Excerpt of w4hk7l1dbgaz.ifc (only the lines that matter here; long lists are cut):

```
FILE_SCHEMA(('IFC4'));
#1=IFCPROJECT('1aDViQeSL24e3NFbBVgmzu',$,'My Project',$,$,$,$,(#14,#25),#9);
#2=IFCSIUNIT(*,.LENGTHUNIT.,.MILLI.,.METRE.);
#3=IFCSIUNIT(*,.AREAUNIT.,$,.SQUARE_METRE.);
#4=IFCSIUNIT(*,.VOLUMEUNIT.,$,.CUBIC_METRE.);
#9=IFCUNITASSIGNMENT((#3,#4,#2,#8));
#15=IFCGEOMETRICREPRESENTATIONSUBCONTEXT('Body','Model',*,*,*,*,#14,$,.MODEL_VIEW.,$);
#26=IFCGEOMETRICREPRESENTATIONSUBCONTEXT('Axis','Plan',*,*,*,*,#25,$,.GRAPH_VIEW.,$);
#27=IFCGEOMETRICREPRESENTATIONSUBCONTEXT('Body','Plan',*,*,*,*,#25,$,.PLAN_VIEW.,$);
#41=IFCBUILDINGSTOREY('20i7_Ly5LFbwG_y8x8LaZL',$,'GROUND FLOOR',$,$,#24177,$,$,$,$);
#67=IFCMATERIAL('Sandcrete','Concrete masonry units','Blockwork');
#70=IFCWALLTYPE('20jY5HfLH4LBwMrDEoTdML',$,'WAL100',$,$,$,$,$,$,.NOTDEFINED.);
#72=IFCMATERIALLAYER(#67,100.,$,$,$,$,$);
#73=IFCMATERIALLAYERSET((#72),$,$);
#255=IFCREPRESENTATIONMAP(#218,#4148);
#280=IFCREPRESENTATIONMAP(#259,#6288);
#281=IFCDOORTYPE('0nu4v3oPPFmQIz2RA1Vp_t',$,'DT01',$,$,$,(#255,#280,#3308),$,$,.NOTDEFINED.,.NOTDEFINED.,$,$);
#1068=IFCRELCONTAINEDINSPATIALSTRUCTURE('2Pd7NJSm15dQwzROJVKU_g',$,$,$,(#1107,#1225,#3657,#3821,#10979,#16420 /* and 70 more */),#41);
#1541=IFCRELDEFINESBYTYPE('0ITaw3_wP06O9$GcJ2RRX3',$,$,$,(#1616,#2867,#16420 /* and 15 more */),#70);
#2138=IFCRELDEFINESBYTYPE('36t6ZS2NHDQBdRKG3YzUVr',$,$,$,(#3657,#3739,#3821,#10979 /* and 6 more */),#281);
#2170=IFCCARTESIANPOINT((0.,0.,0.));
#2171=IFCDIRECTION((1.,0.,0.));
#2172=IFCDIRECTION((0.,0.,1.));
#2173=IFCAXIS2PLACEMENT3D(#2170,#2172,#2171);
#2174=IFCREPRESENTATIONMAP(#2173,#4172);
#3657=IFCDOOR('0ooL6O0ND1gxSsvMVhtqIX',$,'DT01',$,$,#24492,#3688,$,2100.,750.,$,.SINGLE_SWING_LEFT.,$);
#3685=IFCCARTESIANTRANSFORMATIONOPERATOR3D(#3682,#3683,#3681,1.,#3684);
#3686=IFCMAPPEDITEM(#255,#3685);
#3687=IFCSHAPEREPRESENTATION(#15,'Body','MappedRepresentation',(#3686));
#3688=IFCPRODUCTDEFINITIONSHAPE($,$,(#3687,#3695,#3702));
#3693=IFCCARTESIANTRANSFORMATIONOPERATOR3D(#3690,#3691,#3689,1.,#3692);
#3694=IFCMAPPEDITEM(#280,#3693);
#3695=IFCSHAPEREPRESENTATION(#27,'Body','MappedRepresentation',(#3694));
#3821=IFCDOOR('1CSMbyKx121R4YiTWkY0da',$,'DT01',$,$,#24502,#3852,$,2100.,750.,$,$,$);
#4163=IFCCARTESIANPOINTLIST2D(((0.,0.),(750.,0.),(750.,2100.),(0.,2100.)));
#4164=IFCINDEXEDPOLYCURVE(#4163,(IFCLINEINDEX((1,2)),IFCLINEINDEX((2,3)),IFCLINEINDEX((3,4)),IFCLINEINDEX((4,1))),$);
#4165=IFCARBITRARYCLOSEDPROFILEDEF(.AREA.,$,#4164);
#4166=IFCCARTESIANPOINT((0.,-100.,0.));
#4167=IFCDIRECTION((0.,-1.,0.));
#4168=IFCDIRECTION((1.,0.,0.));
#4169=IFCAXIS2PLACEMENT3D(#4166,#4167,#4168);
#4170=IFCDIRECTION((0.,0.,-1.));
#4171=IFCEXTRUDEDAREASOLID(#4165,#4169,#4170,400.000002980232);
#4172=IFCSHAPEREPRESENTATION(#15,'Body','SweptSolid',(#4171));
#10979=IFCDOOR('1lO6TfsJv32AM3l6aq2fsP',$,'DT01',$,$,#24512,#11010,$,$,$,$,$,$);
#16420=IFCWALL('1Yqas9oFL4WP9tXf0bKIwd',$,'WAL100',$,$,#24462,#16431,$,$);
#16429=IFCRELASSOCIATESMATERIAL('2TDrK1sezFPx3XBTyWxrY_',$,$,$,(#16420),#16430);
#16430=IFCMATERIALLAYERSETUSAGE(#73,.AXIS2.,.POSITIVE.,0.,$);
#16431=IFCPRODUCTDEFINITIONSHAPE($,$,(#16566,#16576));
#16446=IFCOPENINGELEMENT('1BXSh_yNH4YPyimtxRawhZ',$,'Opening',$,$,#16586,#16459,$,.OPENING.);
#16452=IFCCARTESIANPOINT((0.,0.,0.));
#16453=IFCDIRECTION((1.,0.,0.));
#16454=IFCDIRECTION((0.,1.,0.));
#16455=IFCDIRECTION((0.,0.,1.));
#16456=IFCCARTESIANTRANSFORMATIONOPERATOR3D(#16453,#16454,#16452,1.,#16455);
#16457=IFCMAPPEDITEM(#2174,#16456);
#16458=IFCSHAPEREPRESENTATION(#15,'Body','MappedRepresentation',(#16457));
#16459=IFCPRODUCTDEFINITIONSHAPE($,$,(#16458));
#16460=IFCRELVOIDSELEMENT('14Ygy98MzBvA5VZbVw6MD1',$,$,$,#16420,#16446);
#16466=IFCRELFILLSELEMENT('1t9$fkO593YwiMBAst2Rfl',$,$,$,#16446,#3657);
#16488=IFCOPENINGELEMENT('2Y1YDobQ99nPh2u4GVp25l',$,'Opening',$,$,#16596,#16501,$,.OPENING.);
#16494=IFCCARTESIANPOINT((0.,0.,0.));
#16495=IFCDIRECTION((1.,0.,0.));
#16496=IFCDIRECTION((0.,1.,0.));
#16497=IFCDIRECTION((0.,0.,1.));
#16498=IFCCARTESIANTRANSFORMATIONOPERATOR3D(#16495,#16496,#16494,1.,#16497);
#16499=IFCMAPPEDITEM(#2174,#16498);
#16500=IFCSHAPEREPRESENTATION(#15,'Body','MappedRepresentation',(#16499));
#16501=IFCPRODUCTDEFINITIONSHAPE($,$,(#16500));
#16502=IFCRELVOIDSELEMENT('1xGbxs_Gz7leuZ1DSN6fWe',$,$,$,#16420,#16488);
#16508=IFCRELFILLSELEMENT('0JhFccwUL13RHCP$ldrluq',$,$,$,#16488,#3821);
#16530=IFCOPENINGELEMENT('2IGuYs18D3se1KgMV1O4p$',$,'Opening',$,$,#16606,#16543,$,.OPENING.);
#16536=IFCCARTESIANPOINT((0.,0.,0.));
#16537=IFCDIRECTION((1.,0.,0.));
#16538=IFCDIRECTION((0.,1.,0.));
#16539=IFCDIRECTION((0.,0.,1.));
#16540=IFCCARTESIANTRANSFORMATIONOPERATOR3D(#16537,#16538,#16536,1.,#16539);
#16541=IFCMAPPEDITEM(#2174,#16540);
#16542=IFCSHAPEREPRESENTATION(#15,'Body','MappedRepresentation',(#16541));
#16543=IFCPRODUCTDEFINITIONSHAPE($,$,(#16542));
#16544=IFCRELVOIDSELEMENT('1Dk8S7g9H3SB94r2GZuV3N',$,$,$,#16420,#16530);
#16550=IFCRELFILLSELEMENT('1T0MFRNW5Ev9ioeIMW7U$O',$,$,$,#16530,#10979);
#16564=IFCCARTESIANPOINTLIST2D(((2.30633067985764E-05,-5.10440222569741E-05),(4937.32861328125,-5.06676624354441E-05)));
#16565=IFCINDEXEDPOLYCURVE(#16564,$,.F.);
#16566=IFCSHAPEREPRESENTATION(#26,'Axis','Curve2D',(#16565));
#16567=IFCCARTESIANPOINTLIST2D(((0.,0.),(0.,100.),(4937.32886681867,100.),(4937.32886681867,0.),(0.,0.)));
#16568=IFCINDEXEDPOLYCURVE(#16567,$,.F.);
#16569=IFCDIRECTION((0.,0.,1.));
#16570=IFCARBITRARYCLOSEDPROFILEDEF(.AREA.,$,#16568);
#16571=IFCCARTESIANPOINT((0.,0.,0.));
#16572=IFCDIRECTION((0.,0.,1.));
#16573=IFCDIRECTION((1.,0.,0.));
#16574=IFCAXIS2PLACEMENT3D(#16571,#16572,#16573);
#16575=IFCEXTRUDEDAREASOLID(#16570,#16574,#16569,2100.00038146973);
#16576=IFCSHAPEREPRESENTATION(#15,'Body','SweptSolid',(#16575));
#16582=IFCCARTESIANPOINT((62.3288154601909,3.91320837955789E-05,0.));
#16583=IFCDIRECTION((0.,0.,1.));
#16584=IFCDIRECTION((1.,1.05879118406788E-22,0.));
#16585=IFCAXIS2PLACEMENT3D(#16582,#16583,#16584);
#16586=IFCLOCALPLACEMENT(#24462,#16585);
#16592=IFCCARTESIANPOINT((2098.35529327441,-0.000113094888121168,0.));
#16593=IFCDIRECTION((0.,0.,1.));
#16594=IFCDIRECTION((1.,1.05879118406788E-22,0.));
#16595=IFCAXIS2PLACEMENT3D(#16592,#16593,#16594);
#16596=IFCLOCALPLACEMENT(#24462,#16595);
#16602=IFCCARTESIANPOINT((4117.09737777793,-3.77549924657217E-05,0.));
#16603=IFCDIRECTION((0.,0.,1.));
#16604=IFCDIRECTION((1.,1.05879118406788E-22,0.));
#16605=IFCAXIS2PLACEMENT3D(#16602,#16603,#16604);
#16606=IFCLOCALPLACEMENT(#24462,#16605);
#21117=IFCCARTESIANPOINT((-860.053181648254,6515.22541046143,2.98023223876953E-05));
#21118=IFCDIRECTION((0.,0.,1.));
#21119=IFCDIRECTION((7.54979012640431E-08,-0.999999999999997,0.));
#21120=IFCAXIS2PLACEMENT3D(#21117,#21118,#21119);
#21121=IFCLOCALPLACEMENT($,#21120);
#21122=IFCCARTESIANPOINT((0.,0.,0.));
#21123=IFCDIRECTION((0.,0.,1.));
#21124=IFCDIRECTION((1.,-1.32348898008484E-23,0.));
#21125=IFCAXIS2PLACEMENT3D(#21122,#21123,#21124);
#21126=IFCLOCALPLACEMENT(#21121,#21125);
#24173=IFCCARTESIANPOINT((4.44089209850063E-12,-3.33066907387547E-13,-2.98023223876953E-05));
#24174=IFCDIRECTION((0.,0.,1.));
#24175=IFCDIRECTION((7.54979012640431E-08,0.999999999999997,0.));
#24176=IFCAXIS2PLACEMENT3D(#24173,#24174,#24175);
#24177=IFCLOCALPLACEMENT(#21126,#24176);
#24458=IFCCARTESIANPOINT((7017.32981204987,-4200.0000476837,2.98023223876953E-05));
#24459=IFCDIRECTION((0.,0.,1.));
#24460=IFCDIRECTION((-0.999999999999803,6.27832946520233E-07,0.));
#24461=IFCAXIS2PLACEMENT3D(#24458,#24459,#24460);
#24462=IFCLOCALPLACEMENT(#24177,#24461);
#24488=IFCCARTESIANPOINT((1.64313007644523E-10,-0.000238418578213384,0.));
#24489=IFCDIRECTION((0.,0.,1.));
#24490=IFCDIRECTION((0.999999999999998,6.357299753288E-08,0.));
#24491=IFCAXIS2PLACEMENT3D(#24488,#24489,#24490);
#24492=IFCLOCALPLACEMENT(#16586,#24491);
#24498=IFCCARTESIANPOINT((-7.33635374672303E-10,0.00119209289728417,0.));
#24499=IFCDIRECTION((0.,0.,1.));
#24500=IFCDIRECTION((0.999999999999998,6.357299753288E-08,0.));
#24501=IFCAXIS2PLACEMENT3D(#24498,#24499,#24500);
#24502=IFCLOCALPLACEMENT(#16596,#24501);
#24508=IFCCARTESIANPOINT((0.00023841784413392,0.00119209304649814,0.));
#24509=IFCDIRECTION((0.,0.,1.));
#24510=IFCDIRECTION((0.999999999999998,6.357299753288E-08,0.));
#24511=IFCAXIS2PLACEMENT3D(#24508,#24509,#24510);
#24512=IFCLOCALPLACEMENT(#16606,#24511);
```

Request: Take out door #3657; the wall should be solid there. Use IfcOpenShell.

```python
import ifcopenshell
import ifcopenshell.api.feature
import ifcopenshell.api.root
import ifcopenshell.geom
import ifcopenshell.util.shape

model = ifcopenshell.open("w4hk7l1dbgaz.ifc")
settings = ifcopenshell.geom.settings()


def volume(element):
    """Net volume in cubic metres, openings subtracted."""
    shape = ifcopenshell.geom.create_shape(settings, element)
    return ifcopenshell.util.shape.get_volume(shape.geometry)


door = model.by_guid("0ooL6O0ND1gxSsvMVhtqIX")
opening = door.FillsVoids[0].RelatingOpeningElement
wall = opening.VoidsElements[0].RelatingBuildingElement
before = volume(wall)

ifcopenshell.api.root.remove_product(model, product=door)
ifcopenshell.api.feature.remove_feature(model, feature=opening)

after = volume(wall)

print(f"wall volume {before:.3f} -> {after:.3f} m3")

model.write("w4hk7l1dbgaz_v2.ifc")
```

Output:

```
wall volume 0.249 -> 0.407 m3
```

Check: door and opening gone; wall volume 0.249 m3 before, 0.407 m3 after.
